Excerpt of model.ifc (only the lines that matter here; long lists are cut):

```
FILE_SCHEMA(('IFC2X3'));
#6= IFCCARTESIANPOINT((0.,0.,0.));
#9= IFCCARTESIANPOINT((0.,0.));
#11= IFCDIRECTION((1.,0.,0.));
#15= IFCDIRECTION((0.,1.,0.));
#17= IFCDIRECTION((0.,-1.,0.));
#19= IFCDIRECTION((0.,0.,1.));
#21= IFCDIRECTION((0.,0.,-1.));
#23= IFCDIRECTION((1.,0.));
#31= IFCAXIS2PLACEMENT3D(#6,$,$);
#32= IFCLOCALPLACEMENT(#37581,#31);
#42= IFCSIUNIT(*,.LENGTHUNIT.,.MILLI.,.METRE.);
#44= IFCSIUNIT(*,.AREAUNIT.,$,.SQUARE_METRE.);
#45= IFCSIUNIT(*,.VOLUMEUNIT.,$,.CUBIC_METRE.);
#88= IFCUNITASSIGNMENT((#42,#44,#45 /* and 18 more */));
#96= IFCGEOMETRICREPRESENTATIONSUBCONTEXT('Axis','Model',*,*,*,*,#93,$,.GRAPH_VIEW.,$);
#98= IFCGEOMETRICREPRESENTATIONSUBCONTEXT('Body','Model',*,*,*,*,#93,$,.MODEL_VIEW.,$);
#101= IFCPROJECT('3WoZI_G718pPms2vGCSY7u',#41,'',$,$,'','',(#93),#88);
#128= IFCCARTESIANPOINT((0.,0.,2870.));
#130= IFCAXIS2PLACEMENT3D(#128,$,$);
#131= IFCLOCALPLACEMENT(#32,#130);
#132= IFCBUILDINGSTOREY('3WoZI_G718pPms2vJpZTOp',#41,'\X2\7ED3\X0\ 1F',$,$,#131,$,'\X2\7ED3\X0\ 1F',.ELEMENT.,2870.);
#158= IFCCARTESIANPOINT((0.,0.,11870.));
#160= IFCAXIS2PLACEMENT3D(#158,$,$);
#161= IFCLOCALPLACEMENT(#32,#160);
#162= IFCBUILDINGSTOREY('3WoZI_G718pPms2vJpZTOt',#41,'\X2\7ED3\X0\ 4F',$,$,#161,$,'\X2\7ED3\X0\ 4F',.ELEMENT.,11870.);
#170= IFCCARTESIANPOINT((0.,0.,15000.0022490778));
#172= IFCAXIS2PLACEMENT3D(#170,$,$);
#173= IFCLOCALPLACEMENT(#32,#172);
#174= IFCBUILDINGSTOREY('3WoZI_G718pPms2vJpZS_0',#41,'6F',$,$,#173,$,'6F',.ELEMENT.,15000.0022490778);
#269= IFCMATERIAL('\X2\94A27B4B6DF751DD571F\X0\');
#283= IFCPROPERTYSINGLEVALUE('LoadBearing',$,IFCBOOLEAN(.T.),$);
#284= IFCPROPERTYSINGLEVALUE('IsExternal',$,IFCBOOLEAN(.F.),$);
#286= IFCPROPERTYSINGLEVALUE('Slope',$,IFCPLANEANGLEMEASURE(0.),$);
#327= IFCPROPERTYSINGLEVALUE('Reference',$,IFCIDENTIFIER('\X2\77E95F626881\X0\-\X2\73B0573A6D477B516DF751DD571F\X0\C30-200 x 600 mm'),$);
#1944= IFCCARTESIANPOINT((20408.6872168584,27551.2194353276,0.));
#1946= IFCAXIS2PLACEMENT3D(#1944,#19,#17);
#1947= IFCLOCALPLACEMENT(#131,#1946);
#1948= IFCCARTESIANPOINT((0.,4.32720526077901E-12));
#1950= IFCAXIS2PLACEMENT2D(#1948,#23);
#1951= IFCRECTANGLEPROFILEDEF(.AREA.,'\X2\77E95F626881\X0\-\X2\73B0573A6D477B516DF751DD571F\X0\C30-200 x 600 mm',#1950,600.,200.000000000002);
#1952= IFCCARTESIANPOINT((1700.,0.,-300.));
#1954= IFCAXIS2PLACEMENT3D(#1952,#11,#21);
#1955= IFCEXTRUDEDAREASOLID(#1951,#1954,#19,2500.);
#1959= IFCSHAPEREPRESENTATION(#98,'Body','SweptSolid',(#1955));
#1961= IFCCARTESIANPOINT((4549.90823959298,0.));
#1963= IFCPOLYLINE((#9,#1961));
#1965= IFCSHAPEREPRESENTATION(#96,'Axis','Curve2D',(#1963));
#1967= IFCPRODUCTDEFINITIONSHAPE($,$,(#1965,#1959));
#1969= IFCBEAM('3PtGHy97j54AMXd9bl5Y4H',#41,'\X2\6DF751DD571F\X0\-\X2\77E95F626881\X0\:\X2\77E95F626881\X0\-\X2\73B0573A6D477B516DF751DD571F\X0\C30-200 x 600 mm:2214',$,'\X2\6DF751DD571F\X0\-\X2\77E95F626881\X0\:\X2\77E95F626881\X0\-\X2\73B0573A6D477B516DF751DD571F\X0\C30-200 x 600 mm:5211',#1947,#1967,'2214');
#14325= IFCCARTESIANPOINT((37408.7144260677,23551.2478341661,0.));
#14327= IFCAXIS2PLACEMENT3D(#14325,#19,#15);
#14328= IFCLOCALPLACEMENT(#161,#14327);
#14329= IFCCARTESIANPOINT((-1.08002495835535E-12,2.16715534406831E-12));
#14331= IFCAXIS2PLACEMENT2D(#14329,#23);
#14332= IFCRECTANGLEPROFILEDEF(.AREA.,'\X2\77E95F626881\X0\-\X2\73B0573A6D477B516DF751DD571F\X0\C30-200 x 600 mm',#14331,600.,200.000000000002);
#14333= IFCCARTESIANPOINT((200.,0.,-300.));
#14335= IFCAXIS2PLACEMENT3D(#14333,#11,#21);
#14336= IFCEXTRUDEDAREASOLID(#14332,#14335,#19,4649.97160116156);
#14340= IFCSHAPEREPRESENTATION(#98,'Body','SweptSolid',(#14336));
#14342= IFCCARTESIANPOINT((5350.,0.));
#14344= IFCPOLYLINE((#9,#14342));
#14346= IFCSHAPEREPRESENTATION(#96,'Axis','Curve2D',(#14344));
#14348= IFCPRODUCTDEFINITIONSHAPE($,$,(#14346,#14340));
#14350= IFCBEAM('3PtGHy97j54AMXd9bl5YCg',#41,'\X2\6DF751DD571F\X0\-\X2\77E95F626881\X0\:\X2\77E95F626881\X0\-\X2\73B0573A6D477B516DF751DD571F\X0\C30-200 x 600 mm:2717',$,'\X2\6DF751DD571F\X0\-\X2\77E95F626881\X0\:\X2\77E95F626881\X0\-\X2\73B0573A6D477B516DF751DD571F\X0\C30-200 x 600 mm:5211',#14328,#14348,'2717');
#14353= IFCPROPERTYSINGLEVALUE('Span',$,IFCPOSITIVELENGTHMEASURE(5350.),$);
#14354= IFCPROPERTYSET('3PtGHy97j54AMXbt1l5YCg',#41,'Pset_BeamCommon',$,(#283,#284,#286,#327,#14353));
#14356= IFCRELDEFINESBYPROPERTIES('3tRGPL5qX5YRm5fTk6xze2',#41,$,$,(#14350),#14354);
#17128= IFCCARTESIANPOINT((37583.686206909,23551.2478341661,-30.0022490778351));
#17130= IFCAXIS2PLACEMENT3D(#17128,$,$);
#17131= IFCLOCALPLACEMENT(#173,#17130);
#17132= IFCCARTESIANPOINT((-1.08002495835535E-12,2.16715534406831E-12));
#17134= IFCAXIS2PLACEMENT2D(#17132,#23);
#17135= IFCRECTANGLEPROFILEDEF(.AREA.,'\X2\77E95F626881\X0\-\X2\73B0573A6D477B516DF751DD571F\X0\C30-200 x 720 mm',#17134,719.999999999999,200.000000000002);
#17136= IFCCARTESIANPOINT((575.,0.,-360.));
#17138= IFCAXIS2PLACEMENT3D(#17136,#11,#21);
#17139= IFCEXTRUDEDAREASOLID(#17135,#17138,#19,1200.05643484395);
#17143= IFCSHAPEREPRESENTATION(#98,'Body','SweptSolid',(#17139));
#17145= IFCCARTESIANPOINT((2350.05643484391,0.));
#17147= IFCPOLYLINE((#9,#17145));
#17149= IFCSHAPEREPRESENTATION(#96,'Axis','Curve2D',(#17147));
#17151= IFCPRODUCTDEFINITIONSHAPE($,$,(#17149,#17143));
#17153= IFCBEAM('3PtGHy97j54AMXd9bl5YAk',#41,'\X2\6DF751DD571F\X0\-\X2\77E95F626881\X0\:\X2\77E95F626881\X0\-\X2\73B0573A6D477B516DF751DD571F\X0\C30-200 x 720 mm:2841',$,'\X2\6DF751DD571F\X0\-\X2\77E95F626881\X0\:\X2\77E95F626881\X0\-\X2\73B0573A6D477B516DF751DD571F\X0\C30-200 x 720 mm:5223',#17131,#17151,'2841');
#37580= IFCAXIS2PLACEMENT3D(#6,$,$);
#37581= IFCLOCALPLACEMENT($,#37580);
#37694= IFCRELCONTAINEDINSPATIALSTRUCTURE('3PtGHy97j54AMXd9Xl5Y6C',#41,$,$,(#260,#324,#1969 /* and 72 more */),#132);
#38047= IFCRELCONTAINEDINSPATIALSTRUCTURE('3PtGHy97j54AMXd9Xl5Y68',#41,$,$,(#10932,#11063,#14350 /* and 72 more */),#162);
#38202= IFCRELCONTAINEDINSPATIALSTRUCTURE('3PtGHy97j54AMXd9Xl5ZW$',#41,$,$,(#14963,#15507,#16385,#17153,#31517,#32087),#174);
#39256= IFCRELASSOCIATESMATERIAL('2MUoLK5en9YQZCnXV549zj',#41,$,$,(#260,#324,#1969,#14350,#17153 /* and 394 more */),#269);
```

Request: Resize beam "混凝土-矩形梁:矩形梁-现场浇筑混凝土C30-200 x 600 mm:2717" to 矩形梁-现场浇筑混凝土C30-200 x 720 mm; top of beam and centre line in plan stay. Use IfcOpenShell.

```python
import ifcopenshell
import ifcopenshell.api.pset
import ifcopenshell.util.element
import ifcopenshell.util.representation

model = ifcopenshell.open("model.ifc")

member = model.by_guid("3PtGHy97j54AMXd9bl5YCg")
source = next(p for p in model.by_type("IfcRectangleProfileDef") if p.ProfileName == "矩形梁-现场浇筑混凝土C30-200 x 720 mm")

body = ifcopenshell.util.representation.get_representation(member, "Model", "Body")
solid = body.Items[0]
old_profile = solid.SweptArea

# Copy the section's sizes but keep this member's own profile position.
profile = ifcopenshell.util.element.copy(model, source)
# Profiles are centred, so shift by half the change in depth to hold the top.
shift = (old_profile.XDim - profile.XDim) / 2
x, y = old_profile.Position.Location.Coordinates
up = (-1.0, 0.0)  # upwards, in the solid's own plane
location = model.createIfcCartesianPoint((x + up[0] * shift, y + up[1] * shift))
profile.Position = model.createIfcAxis2Placement2D(location, old_profile.Position.RefDirection)
solid.SweptArea = profile
if not model.get_total_inverses(old_profile):
    ifcopenshell.util.element.remove_deep2(model, old_profile)
member.Name = member.Name.replace("矩形梁-现场浇筑混凝土C30-200 x 600 mm", "矩形梁-现场浇筑混凝土C30-200 x 720 mm")
member.ObjectType = member.ObjectType.replace("矩形梁-现场浇筑混凝土C30-200 x 600 mm", "矩形梁-现场浇筑混凝土C30-200 x 720 mm")
pset = model.by_id(ifcopenshell.util.element.get_pset(member, "Pset_BeamCommon", should_inherit=False)["id"])
ifcopenshell.api.pset.edit_pset(model, pset=pset, properties={"Reference": "矩形梁-现场浇筑混凝土C30-200 x 720 mm"})

print(solid.SweptArea)

model.write("model_v2.ifc")
```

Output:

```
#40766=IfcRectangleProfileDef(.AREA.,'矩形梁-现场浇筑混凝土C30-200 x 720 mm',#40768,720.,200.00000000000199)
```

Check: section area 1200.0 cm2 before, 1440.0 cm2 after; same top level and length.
